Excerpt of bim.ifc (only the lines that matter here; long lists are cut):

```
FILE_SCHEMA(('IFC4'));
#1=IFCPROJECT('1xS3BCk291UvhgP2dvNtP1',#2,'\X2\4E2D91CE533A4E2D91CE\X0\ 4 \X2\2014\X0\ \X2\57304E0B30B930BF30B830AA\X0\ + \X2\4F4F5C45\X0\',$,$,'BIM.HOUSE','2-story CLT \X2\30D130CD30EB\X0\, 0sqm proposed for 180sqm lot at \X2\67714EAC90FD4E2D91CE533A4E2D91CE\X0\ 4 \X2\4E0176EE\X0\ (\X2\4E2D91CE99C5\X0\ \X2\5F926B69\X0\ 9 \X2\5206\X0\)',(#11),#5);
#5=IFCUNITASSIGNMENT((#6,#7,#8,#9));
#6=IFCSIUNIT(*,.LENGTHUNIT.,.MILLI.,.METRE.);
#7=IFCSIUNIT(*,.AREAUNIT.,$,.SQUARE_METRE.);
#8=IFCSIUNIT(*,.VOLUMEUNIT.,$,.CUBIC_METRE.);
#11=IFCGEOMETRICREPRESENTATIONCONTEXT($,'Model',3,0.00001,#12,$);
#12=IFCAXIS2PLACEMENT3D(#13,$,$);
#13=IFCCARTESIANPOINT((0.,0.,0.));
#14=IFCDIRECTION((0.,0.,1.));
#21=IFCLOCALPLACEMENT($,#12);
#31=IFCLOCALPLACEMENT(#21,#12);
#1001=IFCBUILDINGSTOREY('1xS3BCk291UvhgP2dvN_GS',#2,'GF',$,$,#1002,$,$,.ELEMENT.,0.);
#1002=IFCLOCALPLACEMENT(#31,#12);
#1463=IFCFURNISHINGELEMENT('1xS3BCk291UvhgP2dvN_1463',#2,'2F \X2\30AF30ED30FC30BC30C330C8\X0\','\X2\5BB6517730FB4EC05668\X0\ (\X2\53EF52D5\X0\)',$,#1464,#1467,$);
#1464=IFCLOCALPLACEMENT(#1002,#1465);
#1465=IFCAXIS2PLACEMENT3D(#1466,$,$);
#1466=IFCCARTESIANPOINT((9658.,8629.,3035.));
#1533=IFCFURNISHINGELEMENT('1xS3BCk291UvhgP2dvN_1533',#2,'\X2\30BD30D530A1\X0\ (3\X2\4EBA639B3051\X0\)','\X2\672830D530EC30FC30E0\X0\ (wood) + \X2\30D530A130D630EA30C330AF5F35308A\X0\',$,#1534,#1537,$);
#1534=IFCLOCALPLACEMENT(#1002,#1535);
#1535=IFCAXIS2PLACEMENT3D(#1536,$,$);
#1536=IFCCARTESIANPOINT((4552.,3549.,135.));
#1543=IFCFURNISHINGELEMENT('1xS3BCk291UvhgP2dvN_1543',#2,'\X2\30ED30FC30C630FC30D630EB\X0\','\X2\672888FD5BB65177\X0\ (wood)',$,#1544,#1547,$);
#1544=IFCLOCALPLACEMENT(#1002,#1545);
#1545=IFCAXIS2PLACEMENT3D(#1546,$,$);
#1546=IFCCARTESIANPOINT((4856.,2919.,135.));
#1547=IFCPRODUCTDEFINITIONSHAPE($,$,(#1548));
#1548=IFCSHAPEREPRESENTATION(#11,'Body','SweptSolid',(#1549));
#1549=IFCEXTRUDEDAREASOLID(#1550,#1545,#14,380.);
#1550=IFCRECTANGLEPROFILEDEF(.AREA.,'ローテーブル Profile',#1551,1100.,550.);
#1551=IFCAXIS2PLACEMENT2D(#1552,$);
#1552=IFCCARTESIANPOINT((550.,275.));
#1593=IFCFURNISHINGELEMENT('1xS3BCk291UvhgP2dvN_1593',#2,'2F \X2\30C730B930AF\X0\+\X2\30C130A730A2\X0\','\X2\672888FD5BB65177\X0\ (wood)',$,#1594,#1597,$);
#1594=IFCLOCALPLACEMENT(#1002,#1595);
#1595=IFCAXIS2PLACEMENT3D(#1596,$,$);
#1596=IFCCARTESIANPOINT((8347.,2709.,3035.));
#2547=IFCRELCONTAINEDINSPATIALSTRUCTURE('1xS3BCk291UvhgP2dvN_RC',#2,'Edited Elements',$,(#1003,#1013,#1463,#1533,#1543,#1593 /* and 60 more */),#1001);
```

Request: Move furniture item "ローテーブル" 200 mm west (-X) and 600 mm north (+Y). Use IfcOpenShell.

```python
import ifcopenshell
import ifcopenshell.api.geometry
import ifcopenshell.util.placement
import ifcopenshell.util.unit

model = ifcopenshell.open("bim.ifc")
unit_scale = ifcopenshell.util.unit.calculate_unit_scale(model)

item = model.by_guid("1xS3BCk291UvhgP2dvN_1543")
matrix = ifcopenshell.util.placement.get_local_placement(item.ObjectPlacement)
matrix[0, 3] -= 0.2 / unit_scale
matrix[1, 3] += 0.6 / unit_scale
ifcopenshell.api.geometry.edit_object_placement(model, product=item, matrix=matrix, is_si=False)

print(ifcopenshell.util.placement.get_local_placement(item.ObjectPlacement).round(3) + 0.0)

model.write("bim_rev.ifc")
```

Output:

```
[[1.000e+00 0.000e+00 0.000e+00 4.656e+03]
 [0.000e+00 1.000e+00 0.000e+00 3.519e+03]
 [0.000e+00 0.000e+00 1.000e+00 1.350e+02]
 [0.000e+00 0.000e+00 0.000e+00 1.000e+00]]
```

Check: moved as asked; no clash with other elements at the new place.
